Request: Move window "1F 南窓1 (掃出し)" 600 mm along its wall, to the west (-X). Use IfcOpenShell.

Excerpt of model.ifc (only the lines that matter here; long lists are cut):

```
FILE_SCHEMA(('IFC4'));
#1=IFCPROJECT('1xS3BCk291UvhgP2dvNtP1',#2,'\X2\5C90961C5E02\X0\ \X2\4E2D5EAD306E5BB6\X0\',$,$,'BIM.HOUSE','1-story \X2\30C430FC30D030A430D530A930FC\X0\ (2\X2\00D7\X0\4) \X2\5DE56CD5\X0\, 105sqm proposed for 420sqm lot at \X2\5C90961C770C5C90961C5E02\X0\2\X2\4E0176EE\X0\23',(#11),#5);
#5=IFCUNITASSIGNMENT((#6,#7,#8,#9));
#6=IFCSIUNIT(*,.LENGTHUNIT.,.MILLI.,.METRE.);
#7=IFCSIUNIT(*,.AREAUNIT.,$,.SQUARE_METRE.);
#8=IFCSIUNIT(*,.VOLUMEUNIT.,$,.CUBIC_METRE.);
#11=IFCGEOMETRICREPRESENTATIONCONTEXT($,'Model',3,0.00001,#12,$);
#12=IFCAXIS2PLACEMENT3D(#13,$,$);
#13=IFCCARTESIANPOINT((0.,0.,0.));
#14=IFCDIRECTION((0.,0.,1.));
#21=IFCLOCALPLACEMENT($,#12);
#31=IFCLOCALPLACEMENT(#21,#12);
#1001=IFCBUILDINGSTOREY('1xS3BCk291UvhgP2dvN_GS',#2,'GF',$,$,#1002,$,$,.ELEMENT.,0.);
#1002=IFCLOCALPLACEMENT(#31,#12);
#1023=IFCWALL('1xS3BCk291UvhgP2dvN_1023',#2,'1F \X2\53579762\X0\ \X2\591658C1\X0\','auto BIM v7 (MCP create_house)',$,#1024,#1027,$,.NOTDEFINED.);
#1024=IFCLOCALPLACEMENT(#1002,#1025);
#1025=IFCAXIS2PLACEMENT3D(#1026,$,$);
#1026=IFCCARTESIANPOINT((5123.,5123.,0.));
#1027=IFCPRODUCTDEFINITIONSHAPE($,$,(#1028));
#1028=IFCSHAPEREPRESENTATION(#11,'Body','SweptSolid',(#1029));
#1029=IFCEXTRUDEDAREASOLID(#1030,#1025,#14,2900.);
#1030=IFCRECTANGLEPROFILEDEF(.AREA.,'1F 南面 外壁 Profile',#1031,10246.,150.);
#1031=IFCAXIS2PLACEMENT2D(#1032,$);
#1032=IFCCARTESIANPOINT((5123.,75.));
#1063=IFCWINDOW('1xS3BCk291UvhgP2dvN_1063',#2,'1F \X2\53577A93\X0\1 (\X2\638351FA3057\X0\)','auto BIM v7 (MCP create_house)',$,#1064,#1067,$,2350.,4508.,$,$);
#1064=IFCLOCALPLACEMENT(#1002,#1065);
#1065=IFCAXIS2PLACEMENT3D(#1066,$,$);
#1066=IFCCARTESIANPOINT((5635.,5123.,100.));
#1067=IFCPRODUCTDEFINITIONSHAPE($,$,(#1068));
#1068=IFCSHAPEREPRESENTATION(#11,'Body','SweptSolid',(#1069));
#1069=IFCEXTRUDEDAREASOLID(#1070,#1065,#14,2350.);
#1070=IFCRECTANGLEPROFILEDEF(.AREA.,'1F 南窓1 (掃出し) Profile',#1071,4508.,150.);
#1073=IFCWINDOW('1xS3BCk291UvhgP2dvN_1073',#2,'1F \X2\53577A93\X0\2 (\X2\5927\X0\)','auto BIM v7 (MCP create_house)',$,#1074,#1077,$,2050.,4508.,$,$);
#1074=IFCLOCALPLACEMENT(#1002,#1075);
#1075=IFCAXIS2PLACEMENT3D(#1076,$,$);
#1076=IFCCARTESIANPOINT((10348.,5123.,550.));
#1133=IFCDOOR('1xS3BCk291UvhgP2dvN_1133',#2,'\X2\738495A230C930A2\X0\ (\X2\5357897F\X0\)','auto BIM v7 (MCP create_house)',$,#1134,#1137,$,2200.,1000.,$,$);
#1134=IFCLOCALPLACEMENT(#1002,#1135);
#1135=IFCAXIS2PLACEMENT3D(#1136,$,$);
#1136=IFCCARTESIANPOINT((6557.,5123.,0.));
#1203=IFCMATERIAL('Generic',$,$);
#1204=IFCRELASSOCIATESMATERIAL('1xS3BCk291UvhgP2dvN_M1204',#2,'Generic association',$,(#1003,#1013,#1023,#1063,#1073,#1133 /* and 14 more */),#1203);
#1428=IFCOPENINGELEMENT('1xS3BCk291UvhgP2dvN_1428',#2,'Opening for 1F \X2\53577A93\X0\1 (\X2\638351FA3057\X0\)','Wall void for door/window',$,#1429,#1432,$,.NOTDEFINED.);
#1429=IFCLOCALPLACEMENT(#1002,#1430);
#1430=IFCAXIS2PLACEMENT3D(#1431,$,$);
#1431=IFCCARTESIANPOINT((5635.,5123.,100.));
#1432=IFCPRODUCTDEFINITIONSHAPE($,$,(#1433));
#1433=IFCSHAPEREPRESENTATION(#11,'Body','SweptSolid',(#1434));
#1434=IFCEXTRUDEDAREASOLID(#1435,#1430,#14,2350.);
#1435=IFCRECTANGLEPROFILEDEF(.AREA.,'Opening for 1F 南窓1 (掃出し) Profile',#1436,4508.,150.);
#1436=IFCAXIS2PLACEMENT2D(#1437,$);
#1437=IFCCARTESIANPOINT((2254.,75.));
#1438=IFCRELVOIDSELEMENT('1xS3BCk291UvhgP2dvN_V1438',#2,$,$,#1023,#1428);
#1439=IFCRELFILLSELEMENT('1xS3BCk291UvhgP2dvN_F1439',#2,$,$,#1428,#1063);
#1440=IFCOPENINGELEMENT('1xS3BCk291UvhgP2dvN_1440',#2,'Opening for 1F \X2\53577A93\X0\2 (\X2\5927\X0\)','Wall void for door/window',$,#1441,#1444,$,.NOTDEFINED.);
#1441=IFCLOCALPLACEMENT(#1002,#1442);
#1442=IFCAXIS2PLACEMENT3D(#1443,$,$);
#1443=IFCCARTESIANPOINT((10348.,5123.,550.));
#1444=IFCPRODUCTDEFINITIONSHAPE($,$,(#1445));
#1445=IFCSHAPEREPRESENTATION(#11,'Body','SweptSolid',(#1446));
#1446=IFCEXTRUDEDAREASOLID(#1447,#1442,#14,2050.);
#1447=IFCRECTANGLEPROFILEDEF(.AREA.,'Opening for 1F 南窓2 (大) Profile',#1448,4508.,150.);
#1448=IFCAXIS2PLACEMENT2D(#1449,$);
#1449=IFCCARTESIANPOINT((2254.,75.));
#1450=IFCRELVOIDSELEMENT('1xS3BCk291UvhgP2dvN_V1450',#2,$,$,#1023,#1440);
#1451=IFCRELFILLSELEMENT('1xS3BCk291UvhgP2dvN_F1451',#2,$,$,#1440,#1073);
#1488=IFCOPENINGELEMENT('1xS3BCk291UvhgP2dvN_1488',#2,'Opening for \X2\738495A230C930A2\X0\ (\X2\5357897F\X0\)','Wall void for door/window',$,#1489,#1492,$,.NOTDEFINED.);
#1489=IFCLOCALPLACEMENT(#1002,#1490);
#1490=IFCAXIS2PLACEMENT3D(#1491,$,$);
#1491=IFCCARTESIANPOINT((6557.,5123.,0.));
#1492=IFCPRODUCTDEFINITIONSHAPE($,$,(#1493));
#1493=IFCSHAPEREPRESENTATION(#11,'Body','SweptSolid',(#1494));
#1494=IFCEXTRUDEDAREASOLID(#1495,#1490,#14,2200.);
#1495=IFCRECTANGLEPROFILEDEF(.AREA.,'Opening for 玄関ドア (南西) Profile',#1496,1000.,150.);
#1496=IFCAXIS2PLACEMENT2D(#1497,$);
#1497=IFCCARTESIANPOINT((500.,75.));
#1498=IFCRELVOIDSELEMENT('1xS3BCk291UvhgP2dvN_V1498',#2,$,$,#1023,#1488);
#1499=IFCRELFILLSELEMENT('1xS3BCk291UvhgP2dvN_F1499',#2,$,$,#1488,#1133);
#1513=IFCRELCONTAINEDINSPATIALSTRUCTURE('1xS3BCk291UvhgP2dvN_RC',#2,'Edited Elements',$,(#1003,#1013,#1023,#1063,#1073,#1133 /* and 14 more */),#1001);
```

```python
import ifcopenshell
import ifcopenshell.api.geometry
import ifcopenshell.util.placement
import ifcopenshell.util.unit

model = ifcopenshell.open("model.ifc")
unit_scale = ifcopenshell.util.unit.calculate_unit_scale(model)

window = model.by_id(1063)
opening = window.FillsVoids[0].RelatingOpeningElement
wall = opening.VoidsElements[0].RelatingBuildingElement

wall_matrix = ifcopenshell.util.placement.get_local_placement(wall.ObjectPlacement)
shift = wall_matrix[:3, 0] * -0.6 / unit_scale
before = ifcopenshell.util.placement.get_local_placement(window.ObjectPlacement)[:3, 3].copy()

# The window is not placed relative to its opening, so move both.
for product in (opening, window):
    matrix = ifcopenshell.util.placement.get_local_placement(product.ObjectPlacement)
    matrix[:3, 3] += shift
    ifcopenshell.api.geometry.edit_object_placement(model, product=product, matrix=matrix, is_si=False)

after = ifcopenshell.util.placement.get_local_placement(window.ObjectPlacement)[:3, 3]
print("window moved by", (after - before).round(3) + 0.0)

model.write("model_updated.ifc")
```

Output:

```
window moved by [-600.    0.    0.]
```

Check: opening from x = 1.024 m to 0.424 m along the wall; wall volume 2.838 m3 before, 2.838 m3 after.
